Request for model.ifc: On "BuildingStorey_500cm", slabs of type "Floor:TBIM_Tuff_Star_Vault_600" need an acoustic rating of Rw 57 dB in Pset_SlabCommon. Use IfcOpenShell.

First a look at what the model holds.

```python
import ifcopenshell
import ifcopenshell.util.element

model = ifcopenshell.open("model.ifc")
print(model.schema)
storey = next(s for s in model.by_type("IfcBuildingStorey") if s.Name == "BuildingStorey_500cm")
slabs = [e for e in ifcopenshell.util.element.get_decomposition(storey) if e.is_a("IfcSlab")]
seen = {}
for e in slabs:
    element_type = ifcopenshell.util.element.get_type(e)
    key = (element_type.Name if element_type != e and element_type else None, ifcopenshell.util.element.get_pset(e, "Pset_SlabCommon", "AcousticRating"))
    seen[key] = seen.get(key, 0) + 1
for (name, value), count in sorted(seen.items(), key=str):
    print(count, "x", name, "|", value)
```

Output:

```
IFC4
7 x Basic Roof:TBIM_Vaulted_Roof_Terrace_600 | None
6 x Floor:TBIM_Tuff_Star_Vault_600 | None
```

```python
import ifcopenshell
import ifcopenshell.api.pset
import ifcopenshell.util.element

model = ifcopenshell.open("model.ifc")

storey = next(s for s in model.by_type("IfcBuildingStorey") if s.Name == "BuildingStorey_500cm")
slabs = [e for e in ifcopenshell.util.element.get_decomposition(storey) if e.is_a("IfcSlab")]

count = 0
for e in slabs:
    element_type = ifcopenshell.util.element.get_type(e)
    if element_type in (None, e) or element_type.Name != "Floor:TBIM_Tuff_Star_Vault_600":
        continue
    # add_pset returns the element's existing set when there is one.
    pset = ifcopenshell.api.pset.add_pset(model, product=e, name="Pset_SlabCommon")
    ifcopenshell.api.pset.edit_pset(model, pset=pset, properties={"AcousticRating": "Rw 57 dB"})
    count += 1

print(count, "slabs updated")

model.write("model_v2.ifc")
```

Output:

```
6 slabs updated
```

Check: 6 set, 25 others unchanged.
